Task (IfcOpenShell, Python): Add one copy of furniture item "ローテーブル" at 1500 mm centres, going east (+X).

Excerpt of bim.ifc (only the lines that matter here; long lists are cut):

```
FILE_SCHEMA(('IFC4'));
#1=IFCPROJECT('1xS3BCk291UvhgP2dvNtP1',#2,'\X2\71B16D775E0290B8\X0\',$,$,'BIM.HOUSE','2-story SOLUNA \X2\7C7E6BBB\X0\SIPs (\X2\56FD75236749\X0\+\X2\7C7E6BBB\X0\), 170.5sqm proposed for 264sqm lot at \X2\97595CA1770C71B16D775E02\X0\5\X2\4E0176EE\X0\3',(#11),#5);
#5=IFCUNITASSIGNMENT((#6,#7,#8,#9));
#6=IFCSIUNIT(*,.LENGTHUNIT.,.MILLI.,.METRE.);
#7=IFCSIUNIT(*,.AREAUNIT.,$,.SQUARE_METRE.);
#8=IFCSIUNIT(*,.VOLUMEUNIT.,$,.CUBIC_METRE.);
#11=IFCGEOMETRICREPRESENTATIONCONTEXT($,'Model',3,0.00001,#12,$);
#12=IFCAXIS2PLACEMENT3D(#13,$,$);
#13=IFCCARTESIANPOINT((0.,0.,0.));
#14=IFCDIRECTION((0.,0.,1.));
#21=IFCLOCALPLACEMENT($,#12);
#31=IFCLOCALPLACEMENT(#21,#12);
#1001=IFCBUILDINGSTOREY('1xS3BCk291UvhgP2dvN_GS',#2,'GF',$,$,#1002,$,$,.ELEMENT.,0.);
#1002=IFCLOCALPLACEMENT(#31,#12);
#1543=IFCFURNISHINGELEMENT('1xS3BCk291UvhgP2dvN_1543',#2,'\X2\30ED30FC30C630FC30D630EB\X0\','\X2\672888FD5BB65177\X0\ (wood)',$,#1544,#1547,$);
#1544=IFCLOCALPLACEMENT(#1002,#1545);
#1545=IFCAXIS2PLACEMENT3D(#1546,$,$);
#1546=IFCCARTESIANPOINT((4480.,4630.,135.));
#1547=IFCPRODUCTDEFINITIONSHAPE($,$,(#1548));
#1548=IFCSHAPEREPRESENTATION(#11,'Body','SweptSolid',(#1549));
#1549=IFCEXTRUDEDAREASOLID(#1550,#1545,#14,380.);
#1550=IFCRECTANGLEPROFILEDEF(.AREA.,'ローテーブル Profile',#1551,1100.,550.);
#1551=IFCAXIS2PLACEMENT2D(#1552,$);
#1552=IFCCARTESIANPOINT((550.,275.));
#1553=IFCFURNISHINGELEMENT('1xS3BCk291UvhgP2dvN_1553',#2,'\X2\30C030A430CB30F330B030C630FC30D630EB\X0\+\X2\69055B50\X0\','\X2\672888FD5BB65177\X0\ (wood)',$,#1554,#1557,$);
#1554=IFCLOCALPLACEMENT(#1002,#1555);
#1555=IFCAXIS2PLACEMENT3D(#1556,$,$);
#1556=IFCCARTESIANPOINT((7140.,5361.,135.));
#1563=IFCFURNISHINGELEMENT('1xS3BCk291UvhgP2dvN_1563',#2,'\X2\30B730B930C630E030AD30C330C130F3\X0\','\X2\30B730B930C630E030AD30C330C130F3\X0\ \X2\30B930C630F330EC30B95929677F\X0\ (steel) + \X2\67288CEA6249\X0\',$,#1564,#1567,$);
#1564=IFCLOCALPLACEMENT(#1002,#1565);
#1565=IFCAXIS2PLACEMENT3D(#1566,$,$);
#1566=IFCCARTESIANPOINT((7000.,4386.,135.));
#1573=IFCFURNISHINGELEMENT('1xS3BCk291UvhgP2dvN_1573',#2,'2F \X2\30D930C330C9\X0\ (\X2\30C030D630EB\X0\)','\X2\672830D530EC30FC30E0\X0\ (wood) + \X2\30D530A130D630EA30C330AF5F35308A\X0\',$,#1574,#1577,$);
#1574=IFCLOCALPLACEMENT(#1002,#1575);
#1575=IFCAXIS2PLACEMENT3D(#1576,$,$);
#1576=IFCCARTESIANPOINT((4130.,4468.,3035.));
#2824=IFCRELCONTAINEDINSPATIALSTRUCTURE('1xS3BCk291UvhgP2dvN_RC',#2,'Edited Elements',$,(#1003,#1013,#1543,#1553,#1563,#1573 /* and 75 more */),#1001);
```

```python
import numpy as np
import ifcopenshell
import ifcopenshell.api.geometry
import ifcopenshell.api.root
import ifcopenshell.util.element
import ifcopenshell.util.placement
import ifcopenshell.util.unit

model = ifcopenshell.open("bim.ifc")
unit_scale = ifcopenshell.util.unit.calculate_unit_scale(model)


def reuse_history(source, copy):
    """copy_class also copies each property set's owner history, people and application; keep the originals."""
    for rel in copy.IsDefinedBy:
        if rel.is_a("IfcRelDefinesByProperties") and (history := rel.RelatingPropertyDefinition.OwnerHistory):
            rel.RelatingPropertyDefinition.OwnerHistory = source.OwnerHistory
            ifcopenshell.util.element.remove_deep2(model, history)


source = model.by_guid("1xS3BCk291UvhgP2dvN_1543")
base = ifcopenshell.util.placement.get_local_placement(source.ObjectPlacement)
step = np.array([1.0, 0.0, 0.0]) * 1.5 / unit_scale

for i in range(1, 2):
    copy = ifcopenshell.api.root.copy_class(model, product=source)
    copy.Representation = ifcopenshell.util.element.copy_deep(
        model, source.Representation, exclude=["IfcGeometricRepresentationContext", "IfcRepresentationMap"]
    )
    reuse_history(source, copy)
    matrix = base.copy()
    matrix[:3, 3] += i * step
    print("added at", matrix[:3, 3].round(3) + 0.0)
    ifcopenshell.api.geometry.edit_object_placement(model, product=copy, matrix=matrix, is_si=False)

model.write("bim_edited.ifc")
```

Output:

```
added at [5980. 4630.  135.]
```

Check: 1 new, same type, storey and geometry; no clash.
